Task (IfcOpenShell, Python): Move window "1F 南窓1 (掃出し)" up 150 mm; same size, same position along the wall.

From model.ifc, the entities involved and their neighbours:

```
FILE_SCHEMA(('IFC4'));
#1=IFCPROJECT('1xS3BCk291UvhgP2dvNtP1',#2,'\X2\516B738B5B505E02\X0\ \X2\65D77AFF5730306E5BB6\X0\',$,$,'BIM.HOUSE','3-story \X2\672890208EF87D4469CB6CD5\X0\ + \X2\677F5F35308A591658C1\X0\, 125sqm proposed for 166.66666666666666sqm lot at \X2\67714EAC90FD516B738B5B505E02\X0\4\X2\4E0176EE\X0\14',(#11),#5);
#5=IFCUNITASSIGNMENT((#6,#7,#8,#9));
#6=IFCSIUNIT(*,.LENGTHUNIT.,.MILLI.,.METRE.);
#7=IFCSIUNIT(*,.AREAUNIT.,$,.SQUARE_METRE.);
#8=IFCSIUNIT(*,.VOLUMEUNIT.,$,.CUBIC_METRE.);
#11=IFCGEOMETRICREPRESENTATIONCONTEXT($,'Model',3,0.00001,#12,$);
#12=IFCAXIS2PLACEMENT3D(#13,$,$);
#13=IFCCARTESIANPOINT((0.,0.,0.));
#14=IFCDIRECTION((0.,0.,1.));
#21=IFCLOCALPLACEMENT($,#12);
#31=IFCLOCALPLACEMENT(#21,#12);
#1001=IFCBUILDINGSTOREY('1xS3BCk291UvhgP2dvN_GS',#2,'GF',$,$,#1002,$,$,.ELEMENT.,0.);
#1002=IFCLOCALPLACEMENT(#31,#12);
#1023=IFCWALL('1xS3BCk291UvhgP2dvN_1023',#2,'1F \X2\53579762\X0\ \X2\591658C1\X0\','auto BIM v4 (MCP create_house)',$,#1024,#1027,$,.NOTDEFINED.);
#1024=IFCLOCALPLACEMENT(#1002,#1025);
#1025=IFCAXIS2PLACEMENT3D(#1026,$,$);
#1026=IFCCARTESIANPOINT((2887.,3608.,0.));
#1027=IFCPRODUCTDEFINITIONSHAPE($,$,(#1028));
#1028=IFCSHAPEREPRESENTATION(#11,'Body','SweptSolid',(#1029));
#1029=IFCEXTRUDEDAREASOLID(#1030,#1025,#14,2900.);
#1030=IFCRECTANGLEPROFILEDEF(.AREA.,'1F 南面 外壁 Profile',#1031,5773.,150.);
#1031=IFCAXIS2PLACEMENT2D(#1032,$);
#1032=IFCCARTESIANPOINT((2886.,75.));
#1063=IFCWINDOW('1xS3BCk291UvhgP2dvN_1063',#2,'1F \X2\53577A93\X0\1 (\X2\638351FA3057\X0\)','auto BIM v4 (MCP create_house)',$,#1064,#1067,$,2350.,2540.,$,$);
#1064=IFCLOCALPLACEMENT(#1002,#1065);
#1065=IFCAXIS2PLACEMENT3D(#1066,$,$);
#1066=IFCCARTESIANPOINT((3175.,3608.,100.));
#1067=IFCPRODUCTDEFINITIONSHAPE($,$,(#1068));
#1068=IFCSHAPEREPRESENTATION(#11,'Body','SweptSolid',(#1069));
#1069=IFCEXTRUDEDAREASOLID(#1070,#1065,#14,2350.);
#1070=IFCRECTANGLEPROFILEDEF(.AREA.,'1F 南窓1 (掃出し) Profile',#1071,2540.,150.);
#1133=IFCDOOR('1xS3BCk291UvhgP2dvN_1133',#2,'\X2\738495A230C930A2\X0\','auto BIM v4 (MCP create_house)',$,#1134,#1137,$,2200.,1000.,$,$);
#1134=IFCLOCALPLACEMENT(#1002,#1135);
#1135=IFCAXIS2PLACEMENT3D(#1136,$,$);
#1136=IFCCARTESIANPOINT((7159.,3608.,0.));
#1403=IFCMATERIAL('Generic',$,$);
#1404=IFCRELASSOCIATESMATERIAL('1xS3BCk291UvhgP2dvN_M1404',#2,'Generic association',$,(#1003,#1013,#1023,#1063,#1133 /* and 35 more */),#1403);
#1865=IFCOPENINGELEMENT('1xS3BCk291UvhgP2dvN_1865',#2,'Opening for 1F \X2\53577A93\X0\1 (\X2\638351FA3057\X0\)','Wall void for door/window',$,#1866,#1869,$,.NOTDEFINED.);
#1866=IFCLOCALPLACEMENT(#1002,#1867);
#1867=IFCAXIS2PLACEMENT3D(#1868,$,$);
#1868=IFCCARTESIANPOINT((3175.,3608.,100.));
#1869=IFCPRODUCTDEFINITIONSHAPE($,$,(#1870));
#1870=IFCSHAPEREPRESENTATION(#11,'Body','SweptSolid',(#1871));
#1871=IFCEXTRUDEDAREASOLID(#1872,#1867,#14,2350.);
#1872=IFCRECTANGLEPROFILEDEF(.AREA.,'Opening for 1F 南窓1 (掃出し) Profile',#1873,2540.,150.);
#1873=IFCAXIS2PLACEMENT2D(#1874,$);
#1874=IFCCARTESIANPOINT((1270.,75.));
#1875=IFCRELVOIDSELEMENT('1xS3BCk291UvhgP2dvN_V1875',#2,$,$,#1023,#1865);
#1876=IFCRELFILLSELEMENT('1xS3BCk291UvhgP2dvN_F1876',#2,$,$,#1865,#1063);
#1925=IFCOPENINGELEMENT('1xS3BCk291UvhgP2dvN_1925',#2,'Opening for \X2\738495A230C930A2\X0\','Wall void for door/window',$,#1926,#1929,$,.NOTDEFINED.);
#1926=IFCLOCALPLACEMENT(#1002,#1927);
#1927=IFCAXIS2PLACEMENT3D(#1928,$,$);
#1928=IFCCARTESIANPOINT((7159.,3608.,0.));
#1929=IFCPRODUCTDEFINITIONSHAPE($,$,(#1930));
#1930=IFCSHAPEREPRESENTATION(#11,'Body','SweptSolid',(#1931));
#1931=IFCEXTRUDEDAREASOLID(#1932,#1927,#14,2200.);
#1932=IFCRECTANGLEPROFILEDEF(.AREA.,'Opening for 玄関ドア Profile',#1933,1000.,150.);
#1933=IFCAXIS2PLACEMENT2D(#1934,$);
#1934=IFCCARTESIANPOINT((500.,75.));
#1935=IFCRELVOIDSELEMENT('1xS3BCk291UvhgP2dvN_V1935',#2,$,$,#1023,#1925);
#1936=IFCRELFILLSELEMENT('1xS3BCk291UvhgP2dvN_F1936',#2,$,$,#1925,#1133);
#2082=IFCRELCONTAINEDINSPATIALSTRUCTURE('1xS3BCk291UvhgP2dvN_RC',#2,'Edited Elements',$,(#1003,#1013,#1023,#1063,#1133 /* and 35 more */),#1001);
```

```python
import numpy as np
import ifcopenshell
import ifcopenshell.api.geometry
import ifcopenshell.util.placement
import ifcopenshell.util.unit

model = ifcopenshell.open("model.ifc")
unit_scale = ifcopenshell.util.unit.calculate_unit_scale(model)

window = model.by_guid("1xS3BCk291UvhgP2dvN_1063")
opening = window.FillsVoids[0].RelatingOpeningElement
dz = 0.15 / unit_scale

shift = np.array([0.0, 0.0, dz])
# The window is not placed relative to its opening, so move both.
for product in (opening, window):
    matrix = ifcopenshell.util.placement.get_local_placement(product.ObjectPlacement)
    matrix[:3, 3] += shift
    ifcopenshell.api.geometry.edit_object_placement(model, product=product, matrix=matrix, is_si=False)

print(f"moved by {dz * unit_scale:+.3f} m")

model.write("model_v2.ifc")
```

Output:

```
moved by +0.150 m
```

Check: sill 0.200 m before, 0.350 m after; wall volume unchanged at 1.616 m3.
